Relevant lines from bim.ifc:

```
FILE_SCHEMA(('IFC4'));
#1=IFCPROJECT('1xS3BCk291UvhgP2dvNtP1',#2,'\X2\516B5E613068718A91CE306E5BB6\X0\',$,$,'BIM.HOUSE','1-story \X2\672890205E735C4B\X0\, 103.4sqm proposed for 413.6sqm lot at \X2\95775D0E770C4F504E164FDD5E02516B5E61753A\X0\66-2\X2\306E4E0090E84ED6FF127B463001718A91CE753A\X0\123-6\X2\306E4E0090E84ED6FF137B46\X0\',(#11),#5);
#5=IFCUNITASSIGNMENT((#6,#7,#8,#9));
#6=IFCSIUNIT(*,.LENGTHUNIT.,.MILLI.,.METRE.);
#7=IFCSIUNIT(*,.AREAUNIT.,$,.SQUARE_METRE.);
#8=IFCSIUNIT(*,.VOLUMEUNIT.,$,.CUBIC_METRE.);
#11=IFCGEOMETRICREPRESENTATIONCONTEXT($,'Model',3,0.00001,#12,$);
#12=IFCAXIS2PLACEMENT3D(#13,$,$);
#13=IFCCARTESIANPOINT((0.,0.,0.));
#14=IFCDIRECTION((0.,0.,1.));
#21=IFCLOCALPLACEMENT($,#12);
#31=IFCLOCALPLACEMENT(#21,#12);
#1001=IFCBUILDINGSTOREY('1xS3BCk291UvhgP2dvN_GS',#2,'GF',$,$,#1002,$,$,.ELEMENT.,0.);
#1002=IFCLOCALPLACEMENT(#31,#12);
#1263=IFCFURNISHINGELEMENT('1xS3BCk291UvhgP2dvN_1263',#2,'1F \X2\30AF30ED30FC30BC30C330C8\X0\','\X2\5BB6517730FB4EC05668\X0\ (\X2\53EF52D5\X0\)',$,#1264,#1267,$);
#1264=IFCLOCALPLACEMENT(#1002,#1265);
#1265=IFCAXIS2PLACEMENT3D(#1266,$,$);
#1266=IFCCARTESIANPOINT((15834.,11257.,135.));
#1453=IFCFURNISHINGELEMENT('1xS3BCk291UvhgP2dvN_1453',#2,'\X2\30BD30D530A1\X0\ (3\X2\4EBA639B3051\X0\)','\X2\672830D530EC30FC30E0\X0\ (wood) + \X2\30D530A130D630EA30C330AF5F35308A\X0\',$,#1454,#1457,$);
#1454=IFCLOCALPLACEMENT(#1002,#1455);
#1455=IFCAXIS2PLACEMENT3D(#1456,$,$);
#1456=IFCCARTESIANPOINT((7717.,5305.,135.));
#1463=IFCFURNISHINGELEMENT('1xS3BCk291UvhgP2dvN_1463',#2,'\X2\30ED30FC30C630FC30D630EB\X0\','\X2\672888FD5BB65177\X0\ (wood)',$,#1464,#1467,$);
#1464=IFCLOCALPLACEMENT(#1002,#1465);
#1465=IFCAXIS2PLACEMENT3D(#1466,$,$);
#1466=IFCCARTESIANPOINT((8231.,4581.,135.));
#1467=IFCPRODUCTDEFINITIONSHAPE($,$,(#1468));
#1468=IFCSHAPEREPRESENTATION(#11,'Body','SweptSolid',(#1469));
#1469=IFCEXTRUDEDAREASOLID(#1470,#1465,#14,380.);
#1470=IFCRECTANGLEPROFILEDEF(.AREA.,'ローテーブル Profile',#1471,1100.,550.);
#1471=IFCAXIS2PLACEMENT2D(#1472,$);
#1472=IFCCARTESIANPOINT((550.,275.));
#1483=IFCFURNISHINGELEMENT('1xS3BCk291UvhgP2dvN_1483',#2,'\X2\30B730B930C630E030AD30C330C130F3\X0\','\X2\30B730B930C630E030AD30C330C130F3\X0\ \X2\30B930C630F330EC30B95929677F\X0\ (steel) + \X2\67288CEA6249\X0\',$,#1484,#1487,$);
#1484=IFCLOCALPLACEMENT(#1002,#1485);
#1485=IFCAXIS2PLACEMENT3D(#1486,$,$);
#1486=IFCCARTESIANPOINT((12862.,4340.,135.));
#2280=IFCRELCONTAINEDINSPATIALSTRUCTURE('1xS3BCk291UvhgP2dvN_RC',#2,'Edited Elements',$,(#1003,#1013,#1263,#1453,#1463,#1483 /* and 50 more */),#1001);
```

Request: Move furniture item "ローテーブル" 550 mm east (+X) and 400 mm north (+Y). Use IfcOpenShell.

```python
import ifcopenshell
import ifcopenshell.api.geometry
import ifcopenshell.util.placement

model = ifcopenshell.open("bim.ifc")

item = model.by_guid("1xS3BCk291UvhgP2dvN_1463")
matrix = ifcopenshell.util.placement.get_local_placement(item.ObjectPlacement)
matrix[0, 3] += 550.0
matrix[1, 3] += 400.0
ifcopenshell.api.geometry.edit_object_placement(model, product=item, matrix=matrix, is_si=False)

print(ifcopenshell.util.placement.get_local_placement(item.ObjectPlacement).round(3) + 0.0)

model.write("bim_v2.ifc")
```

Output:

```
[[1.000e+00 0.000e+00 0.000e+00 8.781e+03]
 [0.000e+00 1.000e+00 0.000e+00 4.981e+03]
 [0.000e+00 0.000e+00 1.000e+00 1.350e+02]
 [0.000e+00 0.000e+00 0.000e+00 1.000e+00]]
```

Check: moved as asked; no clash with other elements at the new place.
